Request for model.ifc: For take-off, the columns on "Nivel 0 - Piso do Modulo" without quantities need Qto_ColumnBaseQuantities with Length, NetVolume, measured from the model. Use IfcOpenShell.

First a look at what the model holds.

```python
import ifcopenshell
import ifcopenshell.util.element
import ifcopenshell.util.unit

model = ifcopenshell.open("model.ifc")
print(model.schema)
for unit_type in ("LENGTHUNIT", "AREAUNIT", "VOLUMEUNIT"):
    print(unit_type, ifcopenshell.util.unit.calculate_unit_scale(model, unit_type))
storey = next(s for s in model.by_type("IfcBuildingStorey") if s.Name == "Nivel 0 - Piso do Modulo")
columns = [e for e in ifcopenshell.util.element.get_decomposition(storey) if e.is_a("IfcColumn")]
for e in sorted(columns, key=lambda e: e.id()):
    print(e.id(), e.is_a(), e.Name, list(ifcopenshell.util.element.get_psets(e, qtos_only=True)), sep=" | ")
```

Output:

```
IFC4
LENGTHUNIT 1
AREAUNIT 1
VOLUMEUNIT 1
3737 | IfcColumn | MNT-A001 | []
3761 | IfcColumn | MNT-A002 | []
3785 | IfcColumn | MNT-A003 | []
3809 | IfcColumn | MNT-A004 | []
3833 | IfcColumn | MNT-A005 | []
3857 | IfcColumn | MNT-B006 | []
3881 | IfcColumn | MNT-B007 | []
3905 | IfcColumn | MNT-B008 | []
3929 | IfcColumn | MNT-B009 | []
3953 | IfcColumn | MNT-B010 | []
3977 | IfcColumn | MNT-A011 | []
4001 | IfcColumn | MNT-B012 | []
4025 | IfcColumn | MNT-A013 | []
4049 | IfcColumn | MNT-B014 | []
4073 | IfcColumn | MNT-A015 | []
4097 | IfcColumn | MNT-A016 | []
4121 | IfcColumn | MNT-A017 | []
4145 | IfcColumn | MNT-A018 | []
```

```python
import ifcopenshell
import ifcopenshell.api.pset
import ifcopenshell.geom
import ifcopenshell.util.element
import ifcopenshell.util.shape
import ifcopenshell.util.unit

model = ifcopenshell.open("model.ifc")
unit_scale = ifcopenshell.util.unit.calculate_unit_scale(model)
volume_scale = ifcopenshell.util.unit.calculate_unit_scale(model, "VOLUMEUNIT")
settings = ifcopenshell.geom.settings()

storey = next(s for s in model.by_type("IfcBuildingStorey") if s.Name == "Nivel 0 - Piso do Modulo")
columns = [e for e in ifcopenshell.util.element.get_decomposition(storey) if e.is_a("IfcColumn")]

for e in sorted(columns, key=lambda e: e.id()):
    if ifcopenshell.util.element.get_psets(e, qtos_only=True, should_inherit=False):
        continue
    # Geometry comes back in metres, in the element's own axes.
    shape = ifcopenshell.geom.create_shape(settings, e)
    values = {
        "Length": ifcopenshell.util.shape.get_z(shape.geometry) / unit_scale,
        "NetVolume": ifcopenshell.util.shape.get_volume(shape.geometry) / volume_scale,
    }
    qto = ifcopenshell.api.pset.add_qto(model, product=e, name="Qto_ColumnBaseQuantities")
    ifcopenshell.api.pset.edit_qto(model, qto=qto, properties=values)
    print(e.id(), {k: round(v, 3) for k, v in values.items()})

model.write("model_v2.ifc")
```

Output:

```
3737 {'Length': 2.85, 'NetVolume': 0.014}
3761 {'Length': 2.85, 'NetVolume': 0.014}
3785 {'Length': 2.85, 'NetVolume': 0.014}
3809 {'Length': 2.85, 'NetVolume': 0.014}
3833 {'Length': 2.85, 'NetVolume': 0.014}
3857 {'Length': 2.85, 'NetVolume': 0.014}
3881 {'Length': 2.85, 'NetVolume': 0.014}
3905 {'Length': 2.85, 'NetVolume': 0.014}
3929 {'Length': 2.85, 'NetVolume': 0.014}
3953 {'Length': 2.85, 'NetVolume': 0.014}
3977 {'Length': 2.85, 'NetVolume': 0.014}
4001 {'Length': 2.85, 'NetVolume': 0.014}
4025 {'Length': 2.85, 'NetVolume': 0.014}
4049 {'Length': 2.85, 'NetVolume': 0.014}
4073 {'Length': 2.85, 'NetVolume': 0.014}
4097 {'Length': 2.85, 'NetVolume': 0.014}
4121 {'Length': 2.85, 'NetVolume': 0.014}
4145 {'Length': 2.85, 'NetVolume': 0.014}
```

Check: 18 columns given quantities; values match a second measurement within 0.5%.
